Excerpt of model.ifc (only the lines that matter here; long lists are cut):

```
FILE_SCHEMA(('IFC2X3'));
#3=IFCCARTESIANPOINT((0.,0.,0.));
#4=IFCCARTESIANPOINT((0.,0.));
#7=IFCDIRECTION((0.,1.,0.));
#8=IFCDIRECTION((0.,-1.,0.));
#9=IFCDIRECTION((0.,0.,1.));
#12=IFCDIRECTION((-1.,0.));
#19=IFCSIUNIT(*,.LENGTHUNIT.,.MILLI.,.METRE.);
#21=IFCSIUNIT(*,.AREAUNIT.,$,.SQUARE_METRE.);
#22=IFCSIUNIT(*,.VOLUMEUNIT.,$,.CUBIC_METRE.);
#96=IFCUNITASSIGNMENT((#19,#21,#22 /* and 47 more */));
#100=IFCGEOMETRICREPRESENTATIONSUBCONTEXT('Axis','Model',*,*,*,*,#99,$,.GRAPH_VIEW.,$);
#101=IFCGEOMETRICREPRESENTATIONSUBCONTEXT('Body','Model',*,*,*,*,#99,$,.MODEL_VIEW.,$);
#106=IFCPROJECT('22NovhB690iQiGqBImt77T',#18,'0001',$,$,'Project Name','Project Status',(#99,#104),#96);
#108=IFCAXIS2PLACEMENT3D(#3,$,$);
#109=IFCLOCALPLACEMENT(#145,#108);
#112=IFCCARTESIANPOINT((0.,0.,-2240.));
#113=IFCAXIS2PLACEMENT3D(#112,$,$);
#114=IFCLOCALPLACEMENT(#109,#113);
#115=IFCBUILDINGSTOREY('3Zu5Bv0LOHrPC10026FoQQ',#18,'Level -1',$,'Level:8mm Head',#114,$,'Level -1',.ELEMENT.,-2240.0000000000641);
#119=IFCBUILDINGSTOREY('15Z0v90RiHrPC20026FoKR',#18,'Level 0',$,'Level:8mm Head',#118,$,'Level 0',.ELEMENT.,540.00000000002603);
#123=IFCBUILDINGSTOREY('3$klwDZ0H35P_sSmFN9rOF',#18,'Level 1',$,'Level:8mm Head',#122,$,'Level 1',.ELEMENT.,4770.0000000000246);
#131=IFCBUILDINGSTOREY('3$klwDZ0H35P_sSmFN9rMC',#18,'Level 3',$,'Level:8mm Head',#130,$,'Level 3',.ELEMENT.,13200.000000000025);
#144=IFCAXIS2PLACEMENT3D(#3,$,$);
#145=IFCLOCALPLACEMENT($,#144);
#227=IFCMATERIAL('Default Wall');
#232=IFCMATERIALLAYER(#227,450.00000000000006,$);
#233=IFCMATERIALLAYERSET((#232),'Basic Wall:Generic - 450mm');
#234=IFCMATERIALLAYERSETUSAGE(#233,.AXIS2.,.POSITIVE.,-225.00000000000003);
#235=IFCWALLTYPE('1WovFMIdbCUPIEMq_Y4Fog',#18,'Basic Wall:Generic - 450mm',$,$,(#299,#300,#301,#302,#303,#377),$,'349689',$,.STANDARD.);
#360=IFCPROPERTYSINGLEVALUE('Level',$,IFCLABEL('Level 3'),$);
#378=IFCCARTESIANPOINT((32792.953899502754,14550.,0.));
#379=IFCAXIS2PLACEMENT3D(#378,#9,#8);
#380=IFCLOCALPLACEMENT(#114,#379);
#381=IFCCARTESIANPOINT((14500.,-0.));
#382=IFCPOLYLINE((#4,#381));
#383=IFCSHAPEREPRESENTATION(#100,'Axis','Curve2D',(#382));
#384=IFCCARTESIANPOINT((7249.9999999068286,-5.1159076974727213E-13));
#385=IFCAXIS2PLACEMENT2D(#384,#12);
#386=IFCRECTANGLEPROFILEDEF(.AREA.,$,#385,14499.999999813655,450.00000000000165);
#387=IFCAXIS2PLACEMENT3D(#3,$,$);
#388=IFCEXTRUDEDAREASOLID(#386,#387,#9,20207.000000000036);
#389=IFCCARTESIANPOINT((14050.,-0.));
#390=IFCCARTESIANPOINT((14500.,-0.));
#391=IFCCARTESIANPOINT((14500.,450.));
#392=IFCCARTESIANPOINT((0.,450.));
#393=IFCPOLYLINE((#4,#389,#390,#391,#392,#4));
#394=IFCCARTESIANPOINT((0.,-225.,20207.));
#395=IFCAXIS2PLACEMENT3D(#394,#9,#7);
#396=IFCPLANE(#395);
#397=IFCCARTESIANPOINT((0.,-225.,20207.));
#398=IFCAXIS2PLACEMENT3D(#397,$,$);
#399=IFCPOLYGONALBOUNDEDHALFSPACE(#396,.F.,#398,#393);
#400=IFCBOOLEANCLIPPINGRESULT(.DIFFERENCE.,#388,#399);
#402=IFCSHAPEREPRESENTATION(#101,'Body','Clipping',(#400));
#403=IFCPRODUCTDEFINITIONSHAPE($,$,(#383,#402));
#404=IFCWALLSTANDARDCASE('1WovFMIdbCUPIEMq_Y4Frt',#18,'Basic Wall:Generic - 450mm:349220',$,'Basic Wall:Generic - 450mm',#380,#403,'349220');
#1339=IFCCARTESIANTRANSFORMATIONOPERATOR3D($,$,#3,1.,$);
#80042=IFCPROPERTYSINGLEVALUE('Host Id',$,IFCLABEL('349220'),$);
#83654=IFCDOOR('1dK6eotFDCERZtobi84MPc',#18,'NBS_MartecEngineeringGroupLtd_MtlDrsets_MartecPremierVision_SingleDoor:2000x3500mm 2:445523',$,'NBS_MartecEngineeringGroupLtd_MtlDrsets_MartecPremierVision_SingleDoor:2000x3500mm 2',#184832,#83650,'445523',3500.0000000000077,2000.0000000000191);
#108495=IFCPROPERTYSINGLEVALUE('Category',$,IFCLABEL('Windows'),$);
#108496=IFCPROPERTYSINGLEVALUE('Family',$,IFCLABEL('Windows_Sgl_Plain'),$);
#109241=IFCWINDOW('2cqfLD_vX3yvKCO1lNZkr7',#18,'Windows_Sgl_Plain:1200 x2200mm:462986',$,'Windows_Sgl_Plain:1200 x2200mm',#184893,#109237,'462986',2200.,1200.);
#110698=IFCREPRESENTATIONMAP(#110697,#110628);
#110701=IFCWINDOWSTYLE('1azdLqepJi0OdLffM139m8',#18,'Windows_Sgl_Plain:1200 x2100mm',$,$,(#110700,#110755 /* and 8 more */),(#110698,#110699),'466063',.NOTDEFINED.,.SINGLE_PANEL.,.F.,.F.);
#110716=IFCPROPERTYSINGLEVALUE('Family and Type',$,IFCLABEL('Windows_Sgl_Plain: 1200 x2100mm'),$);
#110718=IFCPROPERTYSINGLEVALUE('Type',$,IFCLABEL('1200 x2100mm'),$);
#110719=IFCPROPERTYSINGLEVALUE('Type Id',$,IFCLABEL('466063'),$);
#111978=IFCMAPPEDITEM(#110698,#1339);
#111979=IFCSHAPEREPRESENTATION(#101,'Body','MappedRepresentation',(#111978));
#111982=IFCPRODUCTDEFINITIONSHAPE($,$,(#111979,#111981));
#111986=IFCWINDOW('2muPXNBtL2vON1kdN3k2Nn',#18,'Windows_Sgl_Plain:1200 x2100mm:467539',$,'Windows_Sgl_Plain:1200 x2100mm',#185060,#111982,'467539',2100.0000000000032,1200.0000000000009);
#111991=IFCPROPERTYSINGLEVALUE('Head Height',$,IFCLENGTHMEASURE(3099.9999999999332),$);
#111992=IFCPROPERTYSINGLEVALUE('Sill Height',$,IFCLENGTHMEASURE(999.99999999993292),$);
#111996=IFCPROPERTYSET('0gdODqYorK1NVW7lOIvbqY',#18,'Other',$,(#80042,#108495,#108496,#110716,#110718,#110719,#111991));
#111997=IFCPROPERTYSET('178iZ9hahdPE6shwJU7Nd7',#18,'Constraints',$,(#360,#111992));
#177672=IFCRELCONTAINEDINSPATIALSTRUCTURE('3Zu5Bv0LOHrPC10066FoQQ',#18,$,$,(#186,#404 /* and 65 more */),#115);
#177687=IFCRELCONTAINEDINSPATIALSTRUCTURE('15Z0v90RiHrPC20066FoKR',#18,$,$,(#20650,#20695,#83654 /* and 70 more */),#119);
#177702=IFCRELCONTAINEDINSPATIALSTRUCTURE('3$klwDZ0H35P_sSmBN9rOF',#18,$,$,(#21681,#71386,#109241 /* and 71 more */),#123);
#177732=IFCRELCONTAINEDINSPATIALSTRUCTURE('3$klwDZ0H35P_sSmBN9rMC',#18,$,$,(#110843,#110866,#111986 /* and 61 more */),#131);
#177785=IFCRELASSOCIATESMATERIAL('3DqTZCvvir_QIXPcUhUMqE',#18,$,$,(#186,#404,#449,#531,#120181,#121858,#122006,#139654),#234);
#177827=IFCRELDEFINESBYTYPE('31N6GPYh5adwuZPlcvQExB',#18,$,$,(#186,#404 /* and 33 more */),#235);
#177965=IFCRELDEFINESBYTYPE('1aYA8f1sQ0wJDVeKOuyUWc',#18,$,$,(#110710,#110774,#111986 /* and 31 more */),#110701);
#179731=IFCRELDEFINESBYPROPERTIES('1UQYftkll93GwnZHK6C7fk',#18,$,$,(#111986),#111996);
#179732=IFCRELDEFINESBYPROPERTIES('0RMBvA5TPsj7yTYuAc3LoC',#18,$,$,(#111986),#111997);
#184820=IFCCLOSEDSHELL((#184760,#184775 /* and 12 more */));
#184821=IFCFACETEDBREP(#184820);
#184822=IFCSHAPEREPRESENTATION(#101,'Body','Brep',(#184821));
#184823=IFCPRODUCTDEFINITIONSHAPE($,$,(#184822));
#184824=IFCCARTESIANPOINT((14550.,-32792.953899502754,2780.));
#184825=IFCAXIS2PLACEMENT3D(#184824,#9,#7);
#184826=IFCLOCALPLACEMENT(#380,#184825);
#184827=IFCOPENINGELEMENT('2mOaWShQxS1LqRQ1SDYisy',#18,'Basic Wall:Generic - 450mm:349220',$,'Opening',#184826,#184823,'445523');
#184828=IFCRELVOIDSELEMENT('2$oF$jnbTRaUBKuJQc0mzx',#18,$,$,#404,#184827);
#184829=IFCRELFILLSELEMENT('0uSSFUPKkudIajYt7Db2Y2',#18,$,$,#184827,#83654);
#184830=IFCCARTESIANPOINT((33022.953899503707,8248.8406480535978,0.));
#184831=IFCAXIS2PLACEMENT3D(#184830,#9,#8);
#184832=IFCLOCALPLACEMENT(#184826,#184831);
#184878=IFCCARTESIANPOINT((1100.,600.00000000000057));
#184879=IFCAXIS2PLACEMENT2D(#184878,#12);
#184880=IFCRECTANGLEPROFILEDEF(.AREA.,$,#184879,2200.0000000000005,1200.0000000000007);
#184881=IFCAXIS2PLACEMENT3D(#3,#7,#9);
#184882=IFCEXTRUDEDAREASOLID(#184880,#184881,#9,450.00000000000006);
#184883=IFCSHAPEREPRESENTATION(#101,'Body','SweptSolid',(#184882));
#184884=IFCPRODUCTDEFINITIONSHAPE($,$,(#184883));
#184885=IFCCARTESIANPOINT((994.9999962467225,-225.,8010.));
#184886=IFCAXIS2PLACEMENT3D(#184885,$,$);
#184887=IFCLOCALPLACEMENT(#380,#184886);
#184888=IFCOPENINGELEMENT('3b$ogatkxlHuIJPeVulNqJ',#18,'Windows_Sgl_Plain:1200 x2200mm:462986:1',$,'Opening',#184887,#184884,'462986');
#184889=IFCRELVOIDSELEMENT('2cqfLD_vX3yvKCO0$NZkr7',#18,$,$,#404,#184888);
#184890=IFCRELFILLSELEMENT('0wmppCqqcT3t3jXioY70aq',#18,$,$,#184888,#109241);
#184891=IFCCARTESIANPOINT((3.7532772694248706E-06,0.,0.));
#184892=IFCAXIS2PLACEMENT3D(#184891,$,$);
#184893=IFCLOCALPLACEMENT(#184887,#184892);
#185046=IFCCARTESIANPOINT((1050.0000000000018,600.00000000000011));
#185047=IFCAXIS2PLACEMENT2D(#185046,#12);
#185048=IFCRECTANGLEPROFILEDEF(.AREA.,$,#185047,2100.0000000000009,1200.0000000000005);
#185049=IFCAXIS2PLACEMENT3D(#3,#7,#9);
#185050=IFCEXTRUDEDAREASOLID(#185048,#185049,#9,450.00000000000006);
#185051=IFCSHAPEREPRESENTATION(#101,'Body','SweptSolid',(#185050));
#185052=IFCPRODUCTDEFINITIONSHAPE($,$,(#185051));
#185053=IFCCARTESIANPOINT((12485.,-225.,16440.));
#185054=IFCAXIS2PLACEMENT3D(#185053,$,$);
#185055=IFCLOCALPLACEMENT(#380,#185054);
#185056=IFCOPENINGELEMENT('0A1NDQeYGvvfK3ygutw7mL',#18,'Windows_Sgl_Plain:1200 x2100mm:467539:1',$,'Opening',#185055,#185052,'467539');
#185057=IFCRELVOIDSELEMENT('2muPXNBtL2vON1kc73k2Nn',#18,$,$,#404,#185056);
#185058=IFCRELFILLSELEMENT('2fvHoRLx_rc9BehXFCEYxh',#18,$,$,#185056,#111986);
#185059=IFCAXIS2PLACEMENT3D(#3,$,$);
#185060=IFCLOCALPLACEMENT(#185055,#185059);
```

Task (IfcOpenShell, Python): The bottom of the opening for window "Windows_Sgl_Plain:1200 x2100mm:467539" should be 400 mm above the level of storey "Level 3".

```python
import numpy as np
import ifcopenshell
import ifcopenshell.api.geometry
import ifcopenshell.api.pset
import ifcopenshell.geom
import ifcopenshell.util.element
import ifcopenshell.util.placement
import ifcopenshell.util.shape
import ifcopenshell.util.unit

model = ifcopenshell.open("model.ifc")
unit_scale = ifcopenshell.util.unit.calculate_unit_scale(model)

window = model.by_guid("2muPXNBtL2vON1kdN3k2Nn")
opening = window.FillsVoids[0].RelatingOpeningElement
storey = ifcopenshell.util.element.get_container(window, ifc_class="IfcBuildingStorey")
level = ifcopenshell.util.placement.get_local_placement(storey.ObjectPlacement)[2, 3]

# The opening's origin need not be at the sill, so measure its lowest point.
shape = ifcopenshell.geom.create_shape(ifcopenshell.geom.settings(), opening)
bottom = ifcopenshell.util.shape.get_shape_bottom_elevation(shape, shape.geometry) / unit_scale
dz = level + 400.0 - bottom

shift = np.array([0.0, 0.0, dz])
# The window is placed relative to its opening, so it follows when the opening moves.
matrix = ifcopenshell.util.placement.get_local_placement(opening.ObjectPlacement)
matrix[:3, 3] += shift
ifcopenshell.api.geometry.edit_object_placement(
    model, product=opening, matrix=matrix, is_si=False, should_transform_children=True
)

# Keep the stored heights in step.
pset = model.by_id(ifcopenshell.util.element.get_pset(window, "Other", should_inherit=False)["id"])
ifcopenshell.api.pset.edit_pset(model, pset=pset, properties={
    "Head Height": model.create_entity("IfcLengthMeasure", ifcopenshell.util.element.get_pset(window, "Other", "Head Height") + dz),
})
pset = model.by_id(ifcopenshell.util.element.get_pset(window, "Constraints", should_inherit=False)["id"])
ifcopenshell.api.pset.edit_pset(model, pset=pset, properties={
    "Sill Height": model.create_entity("IfcLengthMeasure", ifcopenshell.util.element.get_pset(window, "Constraints", "Sill Height") + dz),
})

print(f"moved by {dz * unit_scale:+.3f} m")

model.write("model-out.ifc")
```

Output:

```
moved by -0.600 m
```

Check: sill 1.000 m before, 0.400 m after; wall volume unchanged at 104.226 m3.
